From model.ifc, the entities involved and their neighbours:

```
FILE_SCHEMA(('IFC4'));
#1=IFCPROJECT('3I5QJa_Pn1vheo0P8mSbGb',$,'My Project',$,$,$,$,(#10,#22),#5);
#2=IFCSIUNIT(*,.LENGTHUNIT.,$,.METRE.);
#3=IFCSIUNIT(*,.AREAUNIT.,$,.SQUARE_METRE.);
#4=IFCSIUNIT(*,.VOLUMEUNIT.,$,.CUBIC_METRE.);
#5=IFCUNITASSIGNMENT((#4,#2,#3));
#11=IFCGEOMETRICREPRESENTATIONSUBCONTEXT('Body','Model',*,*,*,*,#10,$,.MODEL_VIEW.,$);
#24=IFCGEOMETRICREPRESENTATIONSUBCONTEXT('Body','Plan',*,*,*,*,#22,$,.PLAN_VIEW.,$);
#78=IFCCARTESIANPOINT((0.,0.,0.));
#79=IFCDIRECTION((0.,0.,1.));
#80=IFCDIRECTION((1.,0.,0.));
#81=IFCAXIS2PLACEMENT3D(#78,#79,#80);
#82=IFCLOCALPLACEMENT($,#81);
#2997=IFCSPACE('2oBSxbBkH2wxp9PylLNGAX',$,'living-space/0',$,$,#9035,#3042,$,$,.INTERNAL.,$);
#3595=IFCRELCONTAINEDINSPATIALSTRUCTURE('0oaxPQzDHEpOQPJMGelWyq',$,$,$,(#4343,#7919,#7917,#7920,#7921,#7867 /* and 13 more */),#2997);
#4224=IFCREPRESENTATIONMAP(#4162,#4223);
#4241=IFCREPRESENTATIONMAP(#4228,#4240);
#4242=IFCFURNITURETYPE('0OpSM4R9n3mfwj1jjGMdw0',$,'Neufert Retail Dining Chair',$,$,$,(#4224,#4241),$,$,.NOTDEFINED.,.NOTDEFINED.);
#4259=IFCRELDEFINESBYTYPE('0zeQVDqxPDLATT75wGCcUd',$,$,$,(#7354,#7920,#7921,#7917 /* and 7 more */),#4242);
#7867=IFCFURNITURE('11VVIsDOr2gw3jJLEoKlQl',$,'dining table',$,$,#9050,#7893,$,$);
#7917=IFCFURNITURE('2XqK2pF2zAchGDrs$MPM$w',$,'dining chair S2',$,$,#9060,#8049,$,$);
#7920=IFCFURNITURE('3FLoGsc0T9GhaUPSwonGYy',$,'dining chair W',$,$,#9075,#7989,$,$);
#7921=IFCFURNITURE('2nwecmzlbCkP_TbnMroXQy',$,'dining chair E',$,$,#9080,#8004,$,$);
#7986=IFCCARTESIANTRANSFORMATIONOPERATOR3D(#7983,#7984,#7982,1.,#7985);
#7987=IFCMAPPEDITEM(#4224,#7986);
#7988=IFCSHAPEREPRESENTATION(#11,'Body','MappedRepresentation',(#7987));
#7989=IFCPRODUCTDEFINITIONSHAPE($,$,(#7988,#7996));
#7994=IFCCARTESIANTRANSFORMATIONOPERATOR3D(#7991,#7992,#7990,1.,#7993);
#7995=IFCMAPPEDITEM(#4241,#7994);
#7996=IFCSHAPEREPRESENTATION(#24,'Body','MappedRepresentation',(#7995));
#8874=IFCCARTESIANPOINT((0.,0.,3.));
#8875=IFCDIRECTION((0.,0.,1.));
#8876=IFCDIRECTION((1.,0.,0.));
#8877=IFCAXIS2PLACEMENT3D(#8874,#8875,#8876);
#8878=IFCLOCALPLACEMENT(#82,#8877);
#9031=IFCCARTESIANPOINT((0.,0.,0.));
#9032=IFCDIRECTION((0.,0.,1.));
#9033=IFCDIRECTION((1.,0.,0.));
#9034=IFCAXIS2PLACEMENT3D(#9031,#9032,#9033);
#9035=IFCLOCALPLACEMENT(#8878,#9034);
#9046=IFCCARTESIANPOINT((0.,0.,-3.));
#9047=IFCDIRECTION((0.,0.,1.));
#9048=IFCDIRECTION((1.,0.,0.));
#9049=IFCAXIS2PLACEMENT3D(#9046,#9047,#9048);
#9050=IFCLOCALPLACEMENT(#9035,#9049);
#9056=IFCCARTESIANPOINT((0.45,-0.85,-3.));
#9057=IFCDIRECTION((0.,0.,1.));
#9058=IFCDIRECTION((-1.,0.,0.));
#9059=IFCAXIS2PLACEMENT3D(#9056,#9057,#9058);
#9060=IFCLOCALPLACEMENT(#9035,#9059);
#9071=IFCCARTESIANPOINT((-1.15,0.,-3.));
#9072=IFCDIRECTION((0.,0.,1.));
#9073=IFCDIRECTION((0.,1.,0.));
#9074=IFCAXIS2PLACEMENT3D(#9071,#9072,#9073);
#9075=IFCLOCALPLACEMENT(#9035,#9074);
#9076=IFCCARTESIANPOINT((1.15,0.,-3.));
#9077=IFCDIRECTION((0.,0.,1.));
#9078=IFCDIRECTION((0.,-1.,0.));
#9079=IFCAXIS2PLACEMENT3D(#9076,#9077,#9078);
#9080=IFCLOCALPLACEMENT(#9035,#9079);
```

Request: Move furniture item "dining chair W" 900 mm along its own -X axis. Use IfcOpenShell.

```python
import ifcopenshell
import ifcopenshell.api.geometry
import ifcopenshell.util.placement
import ifcopenshell.util.unit

model = ifcopenshell.open("model.ifc")
unit_scale = ifcopenshell.util.unit.calculate_unit_scale(model)

item = model.by_guid("3FLoGsc0T9GhaUPSwonGYy")
matrix = ifcopenshell.util.placement.get_local_placement(item.ObjectPlacement)
matrix[:3, 3] -= matrix[:3, 0] * 0.9 / unit_scale
ifcopenshell.api.geometry.edit_object_placement(model, product=item, matrix=matrix, is_si=False)

print(ifcopenshell.util.placement.get_local_placement(item.ObjectPlacement).round(3) + 0.0)

model.write("model_rev.ifc")
```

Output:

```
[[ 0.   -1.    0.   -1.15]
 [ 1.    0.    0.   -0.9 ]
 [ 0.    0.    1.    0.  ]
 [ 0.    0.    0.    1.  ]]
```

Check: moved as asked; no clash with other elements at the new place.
